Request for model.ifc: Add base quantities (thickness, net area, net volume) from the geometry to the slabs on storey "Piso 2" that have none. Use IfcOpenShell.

First a look at what the model holds.

```python
import ifcopenshell
import ifcopenshell.util.element
import ifcopenshell.util.unit

model = ifcopenshell.open("model.ifc")
print(model.schema)
for unit_type in ("LENGTHUNIT", "AREAUNIT", "VOLUMEUNIT"):
    print(unit_type, ifcopenshell.util.unit.calculate_unit_scale(model, unit_type))
storey = next(s for s in model.by_type("IfcBuildingStorey") if s.Name == "Piso 2")
slabs = [e for e in ifcopenshell.util.element.get_decomposition(storey) if e.is_a("IfcSlab")]
for e in sorted(slabs, key=lambda e: e.id()):
    print(e.id(), e.is_a(), e.Name, list(ifcopenshell.util.element.get_psets(e, qtos_only=True)), sep=" | ")
```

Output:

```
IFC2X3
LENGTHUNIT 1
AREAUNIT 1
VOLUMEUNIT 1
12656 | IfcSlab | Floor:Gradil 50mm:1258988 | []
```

```python
import ifcopenshell
import ifcopenshell.api.pset
import ifcopenshell.geom
import ifcopenshell.util.element
import ifcopenshell.util.shape
import ifcopenshell.util.unit

model = ifcopenshell.open("model.ifc")
unit_scale = ifcopenshell.util.unit.calculate_unit_scale(model)
area_scale = ifcopenshell.util.unit.calculate_unit_scale(model, "AREAUNIT")
volume_scale = ifcopenshell.util.unit.calculate_unit_scale(model, "VOLUMEUNIT")
settings = ifcopenshell.geom.settings()

storey = next(s for s in model.by_type("IfcBuildingStorey") if s.Name == "Piso 2")
slabs = [e for e in ifcopenshell.util.element.get_decomposition(storey) if e.is_a("IfcSlab")]

for e in sorted(slabs, key=lambda e: e.id()):
    if ifcopenshell.util.element.get_psets(e, qtos_only=True, should_inherit=False):
        continue
    # Geometry comes back in metres, in the element's own axes.
    shape = ifcopenshell.geom.create_shape(settings, e)
    values = {
        "Width": ifcopenshell.util.shape.get_z(shape.geometry) / unit_scale,
        "NetArea": ifcopenshell.util.shape.get_footprint_area(shape.geometry) / area_scale,
        "NetVolume": ifcopenshell.util.shape.get_volume(shape.geometry) / volume_scale,
    }
    qto = ifcopenshell.api.pset.add_qto(model, product=e, name="BaseQuantities")
    ifcopenshell.api.pset.edit_qto(model, qto=qto, properties=values)
    print(e.id(), {k: round(v, 3) for k, v in values.items()})

model.write("model_edited.ifc")
```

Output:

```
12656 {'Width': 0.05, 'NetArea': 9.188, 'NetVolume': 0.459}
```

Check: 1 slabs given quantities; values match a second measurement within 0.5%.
